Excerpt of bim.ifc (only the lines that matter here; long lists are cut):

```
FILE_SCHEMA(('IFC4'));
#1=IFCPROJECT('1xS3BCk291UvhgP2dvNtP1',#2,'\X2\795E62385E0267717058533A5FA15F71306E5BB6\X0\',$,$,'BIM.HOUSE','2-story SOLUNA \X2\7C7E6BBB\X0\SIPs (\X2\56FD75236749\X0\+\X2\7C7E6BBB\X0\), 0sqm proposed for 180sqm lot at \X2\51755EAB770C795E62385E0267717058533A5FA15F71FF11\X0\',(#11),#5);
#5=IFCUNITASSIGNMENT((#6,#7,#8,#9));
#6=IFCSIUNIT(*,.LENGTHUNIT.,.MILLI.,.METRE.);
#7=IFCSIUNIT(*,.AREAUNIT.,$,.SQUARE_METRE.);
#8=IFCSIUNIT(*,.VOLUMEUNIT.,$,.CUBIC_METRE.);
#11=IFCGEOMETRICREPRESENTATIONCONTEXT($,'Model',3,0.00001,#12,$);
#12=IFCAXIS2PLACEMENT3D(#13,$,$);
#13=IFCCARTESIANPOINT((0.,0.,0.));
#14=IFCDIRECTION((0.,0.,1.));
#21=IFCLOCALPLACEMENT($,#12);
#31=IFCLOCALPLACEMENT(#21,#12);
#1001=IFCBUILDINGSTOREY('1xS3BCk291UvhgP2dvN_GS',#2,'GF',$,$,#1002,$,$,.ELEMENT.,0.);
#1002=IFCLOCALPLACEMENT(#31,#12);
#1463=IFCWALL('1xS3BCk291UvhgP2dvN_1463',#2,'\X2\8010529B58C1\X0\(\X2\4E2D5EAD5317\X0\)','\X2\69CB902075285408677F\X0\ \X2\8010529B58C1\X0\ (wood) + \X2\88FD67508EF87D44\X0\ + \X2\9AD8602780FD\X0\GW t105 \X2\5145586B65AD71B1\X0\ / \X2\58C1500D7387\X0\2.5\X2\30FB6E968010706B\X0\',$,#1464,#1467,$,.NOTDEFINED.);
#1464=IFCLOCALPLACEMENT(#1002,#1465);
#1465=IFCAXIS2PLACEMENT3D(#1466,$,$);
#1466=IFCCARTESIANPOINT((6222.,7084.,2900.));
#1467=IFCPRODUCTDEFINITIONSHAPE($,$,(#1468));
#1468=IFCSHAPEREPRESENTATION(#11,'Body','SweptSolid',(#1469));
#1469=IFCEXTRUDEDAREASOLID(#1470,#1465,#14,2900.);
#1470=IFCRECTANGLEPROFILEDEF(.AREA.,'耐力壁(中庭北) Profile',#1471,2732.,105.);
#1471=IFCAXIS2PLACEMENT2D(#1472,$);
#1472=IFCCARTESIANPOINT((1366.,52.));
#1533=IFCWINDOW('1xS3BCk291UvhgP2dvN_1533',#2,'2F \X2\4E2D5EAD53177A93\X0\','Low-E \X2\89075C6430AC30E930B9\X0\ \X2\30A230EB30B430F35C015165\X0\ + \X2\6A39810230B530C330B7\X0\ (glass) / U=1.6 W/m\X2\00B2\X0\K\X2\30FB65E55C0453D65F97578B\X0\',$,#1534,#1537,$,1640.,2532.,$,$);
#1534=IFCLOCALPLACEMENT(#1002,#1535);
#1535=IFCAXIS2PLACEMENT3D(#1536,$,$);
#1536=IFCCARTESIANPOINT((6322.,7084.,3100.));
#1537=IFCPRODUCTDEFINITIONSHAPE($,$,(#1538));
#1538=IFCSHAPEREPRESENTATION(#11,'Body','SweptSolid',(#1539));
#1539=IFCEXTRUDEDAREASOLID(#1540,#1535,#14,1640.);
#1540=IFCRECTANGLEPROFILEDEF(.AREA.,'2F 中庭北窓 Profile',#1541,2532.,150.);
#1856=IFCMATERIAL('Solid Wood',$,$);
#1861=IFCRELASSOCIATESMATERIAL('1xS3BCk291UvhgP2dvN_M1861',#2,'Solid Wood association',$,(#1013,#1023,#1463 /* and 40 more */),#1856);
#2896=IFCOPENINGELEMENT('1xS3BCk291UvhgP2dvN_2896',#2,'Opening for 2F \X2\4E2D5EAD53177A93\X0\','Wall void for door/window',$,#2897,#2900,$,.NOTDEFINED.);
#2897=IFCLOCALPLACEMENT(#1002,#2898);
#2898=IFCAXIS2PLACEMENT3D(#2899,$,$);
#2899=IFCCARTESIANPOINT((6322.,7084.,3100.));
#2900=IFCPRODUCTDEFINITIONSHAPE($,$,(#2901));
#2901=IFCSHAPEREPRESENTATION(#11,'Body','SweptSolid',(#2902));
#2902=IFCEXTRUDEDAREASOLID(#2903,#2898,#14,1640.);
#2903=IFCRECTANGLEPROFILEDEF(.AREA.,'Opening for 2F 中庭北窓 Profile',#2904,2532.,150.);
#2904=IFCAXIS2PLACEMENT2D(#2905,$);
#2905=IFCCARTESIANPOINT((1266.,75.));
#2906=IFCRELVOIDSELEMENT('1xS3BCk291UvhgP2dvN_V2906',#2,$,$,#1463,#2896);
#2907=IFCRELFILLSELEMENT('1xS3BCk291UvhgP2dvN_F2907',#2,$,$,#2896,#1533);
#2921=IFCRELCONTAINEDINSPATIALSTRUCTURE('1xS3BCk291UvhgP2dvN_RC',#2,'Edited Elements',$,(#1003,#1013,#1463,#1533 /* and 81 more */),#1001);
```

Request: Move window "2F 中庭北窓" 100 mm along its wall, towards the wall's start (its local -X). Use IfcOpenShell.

```python
import ifcopenshell
import ifcopenshell.api.geometry
import ifcopenshell.util.placement

model = ifcopenshell.open("bim.ifc")

window = model.by_id(1533)
opening = window.FillsVoids[0].RelatingOpeningElement
wall = opening.VoidsElements[0].RelatingBuildingElement

wall_matrix = ifcopenshell.util.placement.get_local_placement(wall.ObjectPlacement)
shift = wall_matrix[:3, 0] * -100.0
before = ifcopenshell.util.placement.get_local_placement(window.ObjectPlacement)[:3, 3].copy()

# The window is not placed relative to its opening, so move both.
for product in (opening, window):
    matrix = ifcopenshell.util.placement.get_local_placement(product.ObjectPlacement)
    matrix[:3, 3] += shift
    ifcopenshell.api.geometry.edit_object_placement(model, product=product, matrix=matrix, is_si=False)

after = ifcopenshell.util.placement.get_local_placement(window.ObjectPlacement)[:3, 3]
print("window moved by", (after - before).round(3) + 0.0)

model.write("bim_v2.ifc")
```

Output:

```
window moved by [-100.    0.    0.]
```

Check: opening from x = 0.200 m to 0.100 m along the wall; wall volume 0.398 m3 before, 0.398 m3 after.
